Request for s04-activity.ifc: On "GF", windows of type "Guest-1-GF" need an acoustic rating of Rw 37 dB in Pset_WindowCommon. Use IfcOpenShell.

First a look at what the model holds.

```python
import ifcopenshell
import ifcopenshell.util.element

model = ifcopenshell.open("s04-activity.ifc")
print(model.schema)
storey = next(s for s in model.by_type("IfcBuildingStorey") if s.Name == "GF")
windows = [e for e in ifcopenshell.util.element.get_decomposition(storey) if e.is_a("IfcWindow")]
seen = {}
for e in windows:
    element_type = ifcopenshell.util.element.get_type(e)
    key = (element_type.Name if element_type != e and element_type else None, ifcopenshell.util.element.get_pset(e, "Pset_WindowCommon", "AcousticRating"))
    seen[key] = seen.get(key, 0) + 1
for (name, value), count in sorted(seen.items(), key=str):
    print(count, "x", name, "|", value)
```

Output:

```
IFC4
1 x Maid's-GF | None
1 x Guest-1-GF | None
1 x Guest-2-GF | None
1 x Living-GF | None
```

```python
import ifcopenshell
import ifcopenshell.api.pset
import ifcopenshell.util.element

model = ifcopenshell.open("s04-activity.ifc")

storey = next(s for s in model.by_type("IfcBuildingStorey") if s.Name == "GF")
windows = [e for e in ifcopenshell.util.element.get_decomposition(storey) if e.is_a("IfcWindow")]

count = 0
for e in windows:
    element_type = ifcopenshell.util.element.get_type(e)
    if element_type in (None, e) or element_type.Name != "Guest-1-GF":
        continue
    # add_pset returns the element's existing set when there is one.
    pset = ifcopenshell.api.pset.add_pset(model, product=e, name="Pset_WindowCommon")
    ifcopenshell.api.pset.edit_pset(model, pset=pset, properties={"AcousticRating": "Rw 37 dB"})
    count += 1

print(count, "windows updated")

model.write("s04-activity_v2.ifc")
```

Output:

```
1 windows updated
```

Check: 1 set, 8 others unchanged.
